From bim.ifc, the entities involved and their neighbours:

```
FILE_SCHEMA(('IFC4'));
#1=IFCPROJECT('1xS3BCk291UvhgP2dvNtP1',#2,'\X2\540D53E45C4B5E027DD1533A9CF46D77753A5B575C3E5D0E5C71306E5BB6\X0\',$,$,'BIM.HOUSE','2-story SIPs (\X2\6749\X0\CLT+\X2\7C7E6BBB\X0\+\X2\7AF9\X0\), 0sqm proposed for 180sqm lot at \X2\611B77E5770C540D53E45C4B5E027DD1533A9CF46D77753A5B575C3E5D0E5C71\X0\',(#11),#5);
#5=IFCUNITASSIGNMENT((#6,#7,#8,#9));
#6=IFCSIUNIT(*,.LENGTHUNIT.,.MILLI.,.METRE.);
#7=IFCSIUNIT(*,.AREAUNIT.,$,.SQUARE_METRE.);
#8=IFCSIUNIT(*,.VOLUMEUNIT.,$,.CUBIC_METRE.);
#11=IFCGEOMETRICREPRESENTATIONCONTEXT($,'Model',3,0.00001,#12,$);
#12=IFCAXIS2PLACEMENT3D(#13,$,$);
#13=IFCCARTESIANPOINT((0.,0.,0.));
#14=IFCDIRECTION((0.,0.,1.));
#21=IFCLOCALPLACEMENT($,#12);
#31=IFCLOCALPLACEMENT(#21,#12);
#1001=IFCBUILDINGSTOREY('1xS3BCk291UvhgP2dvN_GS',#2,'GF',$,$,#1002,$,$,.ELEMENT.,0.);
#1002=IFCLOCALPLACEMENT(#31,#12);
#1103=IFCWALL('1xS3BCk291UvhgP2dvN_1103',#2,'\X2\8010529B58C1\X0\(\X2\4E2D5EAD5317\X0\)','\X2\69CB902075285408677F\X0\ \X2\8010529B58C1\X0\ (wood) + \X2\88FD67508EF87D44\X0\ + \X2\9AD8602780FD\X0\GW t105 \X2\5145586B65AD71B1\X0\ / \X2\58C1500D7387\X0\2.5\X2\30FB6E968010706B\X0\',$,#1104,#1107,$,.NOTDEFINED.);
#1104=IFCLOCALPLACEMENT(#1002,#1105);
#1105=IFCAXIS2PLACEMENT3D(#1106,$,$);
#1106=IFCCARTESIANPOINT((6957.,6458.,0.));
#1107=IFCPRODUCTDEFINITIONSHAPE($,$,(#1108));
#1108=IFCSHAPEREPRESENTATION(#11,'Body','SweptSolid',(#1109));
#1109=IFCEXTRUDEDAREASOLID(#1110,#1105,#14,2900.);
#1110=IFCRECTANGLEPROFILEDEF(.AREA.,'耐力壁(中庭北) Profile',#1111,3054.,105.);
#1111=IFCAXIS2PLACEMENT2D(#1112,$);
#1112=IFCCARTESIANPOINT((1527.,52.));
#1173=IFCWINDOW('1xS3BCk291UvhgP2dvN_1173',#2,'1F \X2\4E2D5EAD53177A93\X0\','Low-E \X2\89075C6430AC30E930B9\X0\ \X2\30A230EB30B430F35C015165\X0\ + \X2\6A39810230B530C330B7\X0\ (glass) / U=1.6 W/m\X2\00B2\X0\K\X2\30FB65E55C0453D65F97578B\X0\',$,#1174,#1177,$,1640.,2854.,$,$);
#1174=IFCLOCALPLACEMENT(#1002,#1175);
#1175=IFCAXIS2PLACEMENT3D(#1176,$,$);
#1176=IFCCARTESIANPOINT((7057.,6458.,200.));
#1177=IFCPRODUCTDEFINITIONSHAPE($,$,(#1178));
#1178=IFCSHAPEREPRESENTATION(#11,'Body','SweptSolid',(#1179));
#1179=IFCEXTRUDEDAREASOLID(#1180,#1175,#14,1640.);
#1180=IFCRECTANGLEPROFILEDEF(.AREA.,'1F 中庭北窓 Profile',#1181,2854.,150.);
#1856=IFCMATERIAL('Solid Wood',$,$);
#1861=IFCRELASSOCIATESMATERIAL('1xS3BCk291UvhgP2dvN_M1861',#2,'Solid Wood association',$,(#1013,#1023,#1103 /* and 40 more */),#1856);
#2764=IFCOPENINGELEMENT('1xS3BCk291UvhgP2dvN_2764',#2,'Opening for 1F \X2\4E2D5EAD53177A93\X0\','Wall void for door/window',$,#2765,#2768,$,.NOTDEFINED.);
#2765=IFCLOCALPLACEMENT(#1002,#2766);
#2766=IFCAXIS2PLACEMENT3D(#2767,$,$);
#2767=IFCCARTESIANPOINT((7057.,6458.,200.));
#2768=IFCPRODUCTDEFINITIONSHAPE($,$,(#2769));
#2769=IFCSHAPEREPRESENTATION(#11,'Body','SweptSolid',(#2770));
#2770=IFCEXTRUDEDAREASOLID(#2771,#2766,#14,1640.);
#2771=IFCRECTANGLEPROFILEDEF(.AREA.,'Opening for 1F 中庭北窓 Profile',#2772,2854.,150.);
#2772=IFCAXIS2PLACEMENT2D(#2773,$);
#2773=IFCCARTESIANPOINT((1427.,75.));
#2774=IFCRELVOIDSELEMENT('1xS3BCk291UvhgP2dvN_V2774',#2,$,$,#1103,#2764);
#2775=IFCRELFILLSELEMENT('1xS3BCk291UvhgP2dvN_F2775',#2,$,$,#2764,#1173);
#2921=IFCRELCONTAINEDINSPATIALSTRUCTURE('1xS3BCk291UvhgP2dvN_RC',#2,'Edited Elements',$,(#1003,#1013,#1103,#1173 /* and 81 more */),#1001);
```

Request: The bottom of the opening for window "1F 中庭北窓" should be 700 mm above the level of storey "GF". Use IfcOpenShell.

```python
import numpy as np
import ifcopenshell
import ifcopenshell.api.geometry
import ifcopenshell.geom
import ifcopenshell.util.element
import ifcopenshell.util.placement
import ifcopenshell.util.shape
import ifcopenshell.util.unit

model = ifcopenshell.open("bim.ifc")
unit_scale = ifcopenshell.util.unit.calculate_unit_scale(model)

window = model.by_guid("1xS3BCk291UvhgP2dvN_1173")
opening = window.FillsVoids[0].RelatingOpeningElement
storey = ifcopenshell.util.element.get_container(window, ifc_class="IfcBuildingStorey")
level = ifcopenshell.util.placement.get_local_placement(storey.ObjectPlacement)[2, 3]

# The opening's origin need not be at the sill, so measure its lowest point.
shape = ifcopenshell.geom.create_shape(ifcopenshell.geom.settings(), opening)
bottom = ifcopenshell.util.shape.get_shape_bottom_elevation(shape, shape.geometry) / unit_scale
dz = level + 0.7 / unit_scale - bottom

shift = np.array([0.0, 0.0, dz])
# The window is not placed relative to its opening, so move both.
for product in (opening, window):
    matrix = ifcopenshell.util.placement.get_local_placement(product.ObjectPlacement)
    matrix[:3, 3] += shift
    ifcopenshell.api.geometry.edit_object_placement(model, product=product, matrix=matrix, is_si=False)

print(f"moved by {dz * unit_scale:+.3f} m")

model.write("bim_edited.ifc")
```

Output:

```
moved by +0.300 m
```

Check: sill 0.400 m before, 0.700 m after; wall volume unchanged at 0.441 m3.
